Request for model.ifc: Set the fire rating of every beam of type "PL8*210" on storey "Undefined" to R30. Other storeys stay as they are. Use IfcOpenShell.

First a look at what the model holds.

```python
import ifcopenshell
import ifcopenshell.util.element

model = ifcopenshell.open("model.ifc")
print(model.schema)
storey = next(s for s in model.by_type("IfcBuildingStorey") if s.Name == "Undefined")
beams = [e for e in ifcopenshell.util.element.get_decomposition(storey) if e.is_a("IfcBeam")]
seen = {}
for e in beams:
    element_type = ifcopenshell.util.element.get_type(e)
    key = (element_type.Name if element_type != e and element_type else None, ifcopenshell.util.element.get_pset(e, "Pset_BeamCommon", "FireRating"))
    seen[key] = seen.get(key, 0) + 1
for (name, value), count in sorted(seen.items(), key=str):
    print(count, "x", name, "|", value)
```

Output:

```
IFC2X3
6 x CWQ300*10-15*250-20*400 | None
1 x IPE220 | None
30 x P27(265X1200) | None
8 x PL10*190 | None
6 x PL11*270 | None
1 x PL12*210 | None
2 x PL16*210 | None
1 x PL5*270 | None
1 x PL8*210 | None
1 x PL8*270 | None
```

```python
import ifcopenshell
import ifcopenshell.api.pset
import ifcopenshell.util.element

model = ifcopenshell.open("model.ifc")

storey = next(s for s in model.by_type("IfcBuildingStorey") if s.Name == "Undefined")
beams = [e for e in ifcopenshell.util.element.get_decomposition(storey) if e.is_a("IfcBeam")]

count = 0
for e in beams:
    element_type = ifcopenshell.util.element.get_type(e)
    if element_type in (None, e) or element_type.Name != "PL8*210":
        continue
    found = ifcopenshell.util.element.get_pset(e, "Pset_BeamCommon", should_inherit=False)
    if found:
        pset = model.by_id(found["id"])
        if len(ifcopenshell.util.element.get_elements_by_pset(pset)) > 1:
            pset = ifcopenshell.api.pset.unshare_pset(model, products=[e], pset=pset)[0]
    else:
        pset = ifcopenshell.api.pset.add_pset(model, product=e, name="Pset_BeamCommon")
    ifcopenshell.api.pset.edit_pset(model, pset=pset, properties={"FireRating": "R30"})
    count += 1

print(count, "beams updated")

model.write("model_rev.ifc")
```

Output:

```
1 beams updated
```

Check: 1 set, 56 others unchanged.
